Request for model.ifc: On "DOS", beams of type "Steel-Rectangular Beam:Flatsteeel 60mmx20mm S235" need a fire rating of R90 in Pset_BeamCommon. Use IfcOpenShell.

First a look at what the model holds.

```python
import ifcopenshell
import ifcopenshell.util.element

model = ifcopenshell.open("model.ifc")
print(model.schema)
storey = next(s for s in model.by_type("IfcBuildingStorey") if s.Name == "DOS")
beams = [e for e in ifcopenshell.util.element.get_decomposition(storey) if e.is_a("IfcBeam")]
seen = {}
for e in beams:
    element_type = ifcopenshell.util.element.get_type(e)
    key = (element_type.Name if element_type != e and element_type else None, ifcopenshell.util.element.get_pset(e, "Pset_BeamCommon", "FireRating"))
    seen[key] = seen.get(key, 0) + 1
for (name, value), count in sorted(seen.items(), key=str):
    print(count, "x", name, "|", value)
```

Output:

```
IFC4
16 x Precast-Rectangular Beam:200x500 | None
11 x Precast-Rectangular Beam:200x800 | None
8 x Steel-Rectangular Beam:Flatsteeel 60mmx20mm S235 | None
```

```python
import ifcopenshell
import ifcopenshell.api.pset
import ifcopenshell.util.element

model = ifcopenshell.open("model.ifc")

storey = next(s for s in model.by_type("IfcBuildingStorey") if s.Name == "DOS")
beams = [e for e in ifcopenshell.util.element.get_decomposition(storey) if e.is_a("IfcBeam")]

count = 0
for e in beams:
    element_type = ifcopenshell.util.element.get_type(e)
    if element_type in (None, e) or element_type.Name != "Steel-Rectangular Beam:Flatsteeel 60mmx20mm S235":
        continue
    # add_pset returns the element's existing set when there is one.
    pset = ifcopenshell.api.pset.add_pset(model, product=e, name="Pset_BeamCommon")
    ifcopenshell.api.pset.edit_pset(model, pset=pset, properties={"FireRating": "R90"})
    count += 1

print(count, "beams updated")

model.write("model_edited.ifc")
```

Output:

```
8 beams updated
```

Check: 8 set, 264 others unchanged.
